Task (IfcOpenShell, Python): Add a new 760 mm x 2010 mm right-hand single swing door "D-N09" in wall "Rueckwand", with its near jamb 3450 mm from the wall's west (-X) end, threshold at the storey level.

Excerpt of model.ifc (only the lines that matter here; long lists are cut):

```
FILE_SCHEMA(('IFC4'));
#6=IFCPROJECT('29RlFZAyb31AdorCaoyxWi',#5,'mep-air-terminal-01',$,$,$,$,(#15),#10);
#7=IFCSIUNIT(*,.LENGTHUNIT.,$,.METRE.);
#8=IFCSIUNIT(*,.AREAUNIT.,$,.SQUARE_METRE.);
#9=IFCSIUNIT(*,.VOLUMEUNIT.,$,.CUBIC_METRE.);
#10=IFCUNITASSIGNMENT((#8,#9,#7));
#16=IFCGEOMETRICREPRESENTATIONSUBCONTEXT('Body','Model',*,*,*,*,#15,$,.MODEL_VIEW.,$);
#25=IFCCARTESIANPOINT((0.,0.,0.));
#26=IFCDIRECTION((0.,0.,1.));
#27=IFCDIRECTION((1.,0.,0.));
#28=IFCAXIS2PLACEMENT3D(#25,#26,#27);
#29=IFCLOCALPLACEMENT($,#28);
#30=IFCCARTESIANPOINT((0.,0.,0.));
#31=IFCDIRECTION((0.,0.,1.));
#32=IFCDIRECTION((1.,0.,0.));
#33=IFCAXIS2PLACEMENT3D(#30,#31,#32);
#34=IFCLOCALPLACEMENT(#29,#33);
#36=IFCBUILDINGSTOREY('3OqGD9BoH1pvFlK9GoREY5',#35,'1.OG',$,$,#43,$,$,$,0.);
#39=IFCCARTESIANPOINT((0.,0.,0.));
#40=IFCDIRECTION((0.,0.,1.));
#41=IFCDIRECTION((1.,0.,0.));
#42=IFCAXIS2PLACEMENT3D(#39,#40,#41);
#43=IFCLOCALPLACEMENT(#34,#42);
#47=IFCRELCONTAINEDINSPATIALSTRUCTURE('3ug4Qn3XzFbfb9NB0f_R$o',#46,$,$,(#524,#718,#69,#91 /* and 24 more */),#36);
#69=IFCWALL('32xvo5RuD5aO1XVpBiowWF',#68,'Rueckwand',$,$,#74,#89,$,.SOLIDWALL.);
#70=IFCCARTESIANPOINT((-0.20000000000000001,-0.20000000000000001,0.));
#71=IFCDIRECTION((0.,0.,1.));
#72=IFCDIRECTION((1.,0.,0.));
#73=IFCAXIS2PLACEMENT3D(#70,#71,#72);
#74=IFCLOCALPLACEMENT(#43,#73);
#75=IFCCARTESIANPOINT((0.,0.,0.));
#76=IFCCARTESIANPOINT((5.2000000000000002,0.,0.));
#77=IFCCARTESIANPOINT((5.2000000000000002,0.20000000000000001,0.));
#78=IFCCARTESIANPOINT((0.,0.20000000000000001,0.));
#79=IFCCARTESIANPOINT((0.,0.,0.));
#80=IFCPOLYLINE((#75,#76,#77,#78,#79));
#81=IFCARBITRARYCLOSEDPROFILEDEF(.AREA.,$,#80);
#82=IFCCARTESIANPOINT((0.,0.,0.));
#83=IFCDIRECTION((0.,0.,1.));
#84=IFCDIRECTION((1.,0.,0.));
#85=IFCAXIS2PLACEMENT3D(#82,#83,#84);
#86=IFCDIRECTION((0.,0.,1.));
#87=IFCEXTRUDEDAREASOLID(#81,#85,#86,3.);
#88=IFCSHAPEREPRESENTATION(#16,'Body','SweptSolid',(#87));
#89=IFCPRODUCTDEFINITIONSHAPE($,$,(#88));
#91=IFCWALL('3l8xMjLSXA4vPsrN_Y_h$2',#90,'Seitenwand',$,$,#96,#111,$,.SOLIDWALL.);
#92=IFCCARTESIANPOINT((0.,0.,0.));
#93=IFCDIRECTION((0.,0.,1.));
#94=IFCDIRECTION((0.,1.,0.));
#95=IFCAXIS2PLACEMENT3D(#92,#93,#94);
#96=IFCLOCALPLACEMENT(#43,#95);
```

```python
import numpy as np
import ifcopenshell
import ifcopenshell.api.feature
import ifcopenshell.api.geometry
import ifcopenshell.api.root
import ifcopenshell.api.spatial
import ifcopenshell.geom
import ifcopenshell.util.element
import ifcopenshell.util.placement
import ifcopenshell.util.representation
import ifcopenshell.util.shape
import ifcopenshell.util.unit

model = ifcopenshell.open("model.ifc")
unit_scale = ifcopenshell.util.unit.calculate_unit_scale(model)
settings = ifcopenshell.geom.settings()


def volume(element):
    """Net volume in cubic metres, openings subtracted."""
    shape = ifcopenshell.geom.create_shape(settings, element)
    return ifcopenshell.util.shape.get_volume(shape.geometry)


wall = model.by_id(69)
storey = ifcopenshell.util.element.get_container(wall, ifc_class="IfcBuildingStorey")
context = ifcopenshell.util.representation.get_context(model, "Model", "Body", "MODEL_VIEW")
before = volume(wall)

width, height, from_end, sill = 0.76, 2.01, 3.45, 0.0  # metres

# The wall runs along its own X axis, and the end named is its -X end.
wall_shape = ifcopenshell.geom.create_shape(settings, wall)
x, y, z = ifcopenshell.util.shape.get_vertices(wall_shape.geometry).T
start = x.min() + from_end
face, thickness = float(y.min()), float(y.max() - y.min())
wall_matrix = ifcopenshell.util.placement.get_local_placement(wall.ObjectPlacement)
level = ifcopenshell.util.placement.get_local_placement(storey.ObjectPlacement)[2, 3]


def in_wall(x, y):
    """Placement at x, y metres in the wall's axes, at sill height."""
    matrix = wall_matrix.copy()
    matrix[:, 3] = wall_matrix @ np.array([x / unit_scale, y / unit_scale, 0.0, 1.0])
    matrix[2, 3] = level + sill / unit_scale
    return matrix


# Opening: a box that overshoots both wall faces by 50 mm.
opening = ifcopenshell.api.root.create_entity(model, ifc_class="IfcOpeningElement", predefined_type="OPENING")
box = ifcopenshell.api.geometry.add_wall_representation(
    model, context=context, length=width, height=height, thickness=thickness + 0.1
)
ifcopenshell.api.geometry.assign_representation(model, product=opening, representation=box)
ifcopenshell.api.geometry.edit_object_placement(model, product=opening, matrix=in_wall(start, face - 0.05), is_si=False)
ifcopenshell.api.feature.add_feature(model, feature=opening, element=wall)

door = ifcopenshell.api.root.create_entity(model, ifc_class="IfcDoor", name="D-N09", predefined_type="DOOR")
door.OverallWidth, door.OverallHeight = width / unit_scale, height / unit_scale
door.OperationType = "SINGLE_SWING_RIGHT"
body = ifcopenshell.api.geometry.add_door_representation(
    model,
    context=context,
    overall_width=door.OverallWidth,
    overall_height=door.OverallHeight,
    operation_type="SINGLE_SWING_RIGHT",
    lining_properties={"LiningDepth": thickness / unit_scale, "ThresholdDepth": thickness / unit_scale},
)
ifcopenshell.api.geometry.assign_representation(model, product=door, representation=body)
ifcopenshell.api.spatial.assign_container(model, products=[door], relating_structure=storey)
ifcopenshell.api.feature.add_filling(model, opening=opening, element=door)

# The lining spans the wall, so the door starts at the wall face.
ifcopenshell.api.geometry.edit_object_placement(model, product=door, matrix=in_wall(start, face), is_si=False)

after = volume(wall)

print(f"wall volume {before:.3f} -> {after:.3f} m3")

model.write("model_v2.ifc")
```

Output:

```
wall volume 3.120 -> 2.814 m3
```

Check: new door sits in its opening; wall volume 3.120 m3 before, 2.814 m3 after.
